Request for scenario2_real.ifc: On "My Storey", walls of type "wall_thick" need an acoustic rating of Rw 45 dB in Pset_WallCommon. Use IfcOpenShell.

First a look at what the model holds.

```python
import ifcopenshell
import ifcopenshell.util.element

model = ifcopenshell.open("scenario2_real.ifc")
print(model.schema)
storey = next(s for s in model.by_type("IfcBuildingStorey") if s.Name == "My Storey")
walls = [e for e in ifcopenshell.util.element.get_decomposition(storey) if e.is_a("IfcWall")]
seen = {}
for e in walls:
    element_type = ifcopenshell.util.element.get_type(e)
    key = (element_type.Name if element_type != e and element_type else None, ifcopenshell.util.element.get_pset(e, "Pset_WallCommon", "AcousticRating"))
    seen[key] = seen.get(key, 0) + 1
for (name, value), count in sorted(seen.items(), key=str):
    print(count, "x", name, "|", value)
```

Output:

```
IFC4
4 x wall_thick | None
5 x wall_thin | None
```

```python
import ifcopenshell
import ifcopenshell.api.pset
import ifcopenshell.util.element

model = ifcopenshell.open("scenario2_real.ifc")

storey = next(s for s in model.by_type("IfcBuildingStorey") if s.Name == "My Storey")
walls = [e for e in ifcopenshell.util.element.get_decomposition(storey) if e.is_a("IfcWall")]

count = 0
for e in walls:
    element_type = ifcopenshell.util.element.get_type(e)
    if element_type in (None, e) or element_type.Name != "wall_thick":
        continue
    # add_pset returns the element's existing set when there is one.
    pset = ifcopenshell.api.pset.add_pset(model, product=e, name="Pset_WallCommon")
    ifcopenshell.api.pset.edit_pset(model, pset=pset, properties={"AcousticRating": "Rw 45 dB"})
    count += 1

print(count, "walls updated")

model.write("scenario2_real_updated.ifc")
```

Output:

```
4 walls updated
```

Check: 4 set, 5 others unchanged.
